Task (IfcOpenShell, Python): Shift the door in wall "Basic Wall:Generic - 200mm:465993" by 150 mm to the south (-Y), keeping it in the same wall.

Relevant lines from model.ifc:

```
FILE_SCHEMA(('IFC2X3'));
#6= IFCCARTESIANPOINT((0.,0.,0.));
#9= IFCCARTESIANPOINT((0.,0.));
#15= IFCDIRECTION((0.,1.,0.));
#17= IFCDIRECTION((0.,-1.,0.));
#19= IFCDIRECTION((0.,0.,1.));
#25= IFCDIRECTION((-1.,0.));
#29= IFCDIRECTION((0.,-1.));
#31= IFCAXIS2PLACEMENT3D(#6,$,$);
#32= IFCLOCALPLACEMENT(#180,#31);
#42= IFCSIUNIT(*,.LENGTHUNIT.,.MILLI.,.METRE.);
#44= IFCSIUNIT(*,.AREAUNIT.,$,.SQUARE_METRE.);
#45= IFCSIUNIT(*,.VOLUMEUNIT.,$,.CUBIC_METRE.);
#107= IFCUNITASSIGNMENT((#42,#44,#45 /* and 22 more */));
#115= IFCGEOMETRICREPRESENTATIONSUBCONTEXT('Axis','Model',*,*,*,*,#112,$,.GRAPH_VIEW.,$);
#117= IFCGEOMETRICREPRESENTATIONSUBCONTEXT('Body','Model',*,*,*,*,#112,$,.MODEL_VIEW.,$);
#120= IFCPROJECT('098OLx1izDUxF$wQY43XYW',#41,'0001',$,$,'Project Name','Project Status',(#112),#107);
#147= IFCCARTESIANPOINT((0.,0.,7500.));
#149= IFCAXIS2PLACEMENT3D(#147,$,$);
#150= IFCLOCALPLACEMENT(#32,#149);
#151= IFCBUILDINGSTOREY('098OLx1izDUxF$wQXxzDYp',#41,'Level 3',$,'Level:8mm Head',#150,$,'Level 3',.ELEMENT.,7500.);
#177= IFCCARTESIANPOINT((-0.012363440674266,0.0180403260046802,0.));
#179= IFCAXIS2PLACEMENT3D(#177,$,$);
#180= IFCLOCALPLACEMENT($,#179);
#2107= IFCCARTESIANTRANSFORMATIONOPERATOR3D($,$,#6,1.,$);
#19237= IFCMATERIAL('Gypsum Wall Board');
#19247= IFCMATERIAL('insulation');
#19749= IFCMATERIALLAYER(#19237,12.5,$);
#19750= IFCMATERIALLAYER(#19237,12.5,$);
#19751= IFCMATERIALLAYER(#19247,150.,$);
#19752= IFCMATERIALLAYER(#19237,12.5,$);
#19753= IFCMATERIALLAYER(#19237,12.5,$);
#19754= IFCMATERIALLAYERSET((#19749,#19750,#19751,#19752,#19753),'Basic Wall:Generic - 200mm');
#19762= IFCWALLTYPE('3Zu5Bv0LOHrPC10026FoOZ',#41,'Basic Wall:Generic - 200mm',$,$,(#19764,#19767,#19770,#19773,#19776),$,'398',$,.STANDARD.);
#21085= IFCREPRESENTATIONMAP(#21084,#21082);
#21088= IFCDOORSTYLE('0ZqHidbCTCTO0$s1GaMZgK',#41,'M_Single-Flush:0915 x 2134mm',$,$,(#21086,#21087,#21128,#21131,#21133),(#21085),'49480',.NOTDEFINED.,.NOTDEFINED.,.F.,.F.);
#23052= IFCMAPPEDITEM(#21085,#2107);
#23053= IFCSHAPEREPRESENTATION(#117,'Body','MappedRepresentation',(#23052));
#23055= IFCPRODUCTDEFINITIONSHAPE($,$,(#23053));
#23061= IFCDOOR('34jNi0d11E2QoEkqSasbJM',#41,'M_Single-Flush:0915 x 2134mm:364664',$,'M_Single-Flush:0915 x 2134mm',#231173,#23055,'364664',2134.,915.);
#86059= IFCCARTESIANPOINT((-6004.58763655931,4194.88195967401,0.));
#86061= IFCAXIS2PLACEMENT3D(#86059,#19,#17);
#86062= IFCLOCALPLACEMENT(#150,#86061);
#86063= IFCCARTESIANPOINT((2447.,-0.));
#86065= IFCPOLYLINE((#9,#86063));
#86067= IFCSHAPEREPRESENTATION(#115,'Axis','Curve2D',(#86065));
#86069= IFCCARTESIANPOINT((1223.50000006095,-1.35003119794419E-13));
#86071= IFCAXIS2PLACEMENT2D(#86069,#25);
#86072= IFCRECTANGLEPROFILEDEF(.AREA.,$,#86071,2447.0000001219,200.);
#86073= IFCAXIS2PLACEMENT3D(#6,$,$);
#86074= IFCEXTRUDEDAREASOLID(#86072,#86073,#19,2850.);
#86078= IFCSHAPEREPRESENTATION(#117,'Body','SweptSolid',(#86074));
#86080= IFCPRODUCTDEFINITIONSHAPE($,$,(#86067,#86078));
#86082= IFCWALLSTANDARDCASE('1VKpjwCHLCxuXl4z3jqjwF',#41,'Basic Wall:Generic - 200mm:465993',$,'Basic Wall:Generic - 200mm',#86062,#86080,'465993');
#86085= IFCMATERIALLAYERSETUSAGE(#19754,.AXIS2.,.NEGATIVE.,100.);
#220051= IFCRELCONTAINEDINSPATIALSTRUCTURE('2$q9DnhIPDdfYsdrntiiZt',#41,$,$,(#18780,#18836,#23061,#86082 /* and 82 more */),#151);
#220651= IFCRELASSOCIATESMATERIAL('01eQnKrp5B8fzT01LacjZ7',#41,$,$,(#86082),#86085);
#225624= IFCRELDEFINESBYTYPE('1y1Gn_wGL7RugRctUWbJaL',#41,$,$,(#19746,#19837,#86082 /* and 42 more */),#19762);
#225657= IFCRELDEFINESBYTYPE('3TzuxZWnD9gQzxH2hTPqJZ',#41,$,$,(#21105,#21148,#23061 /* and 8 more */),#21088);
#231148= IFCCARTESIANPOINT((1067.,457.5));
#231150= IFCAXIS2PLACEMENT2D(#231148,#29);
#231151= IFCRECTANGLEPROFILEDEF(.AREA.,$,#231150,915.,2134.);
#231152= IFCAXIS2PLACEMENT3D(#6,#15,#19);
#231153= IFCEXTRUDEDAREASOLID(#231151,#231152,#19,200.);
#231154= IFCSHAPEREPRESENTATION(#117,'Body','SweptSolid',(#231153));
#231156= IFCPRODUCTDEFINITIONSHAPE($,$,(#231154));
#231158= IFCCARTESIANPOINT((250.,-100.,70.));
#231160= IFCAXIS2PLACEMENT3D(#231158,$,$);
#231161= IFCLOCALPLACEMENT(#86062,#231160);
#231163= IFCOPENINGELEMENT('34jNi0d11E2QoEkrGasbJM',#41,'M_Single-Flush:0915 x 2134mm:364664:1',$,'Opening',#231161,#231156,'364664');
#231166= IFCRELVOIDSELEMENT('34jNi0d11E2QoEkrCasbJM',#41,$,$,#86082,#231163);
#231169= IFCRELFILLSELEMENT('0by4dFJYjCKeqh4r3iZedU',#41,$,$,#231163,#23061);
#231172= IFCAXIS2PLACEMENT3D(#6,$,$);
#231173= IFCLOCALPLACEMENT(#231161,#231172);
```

```python
import ifcopenshell
import ifcopenshell.api.geometry
import ifcopenshell.util.placement
import ifcopenshell.util.unit

model = ifcopenshell.open("model.ifc")
unit_scale = ifcopenshell.util.unit.calculate_unit_scale(model)

door = model.by_guid("34jNi0d11E2QoEkqSasbJM")
opening = door.FillsVoids[0].RelatingOpeningElement
wall = opening.VoidsElements[0].RelatingBuildingElement

wall_matrix = ifcopenshell.util.placement.get_local_placement(wall.ObjectPlacement)
shift = wall_matrix[:3, 0] * 0.15 / unit_scale
before = ifcopenshell.util.placement.get_local_placement(door.ObjectPlacement)[:3, 3].copy()

# The door is placed relative to its opening, so it follows when the opening moves.
matrix = ifcopenshell.util.placement.get_local_placement(opening.ObjectPlacement)
matrix[:3, 3] += shift
ifcopenshell.api.geometry.edit_object_placement(
    model, product=opening, matrix=matrix, is_si=False, should_transform_children=True
)

after = ifcopenshell.util.placement.get_local_placement(door.ObjectPlacement)[:3, 3]
print("door moved by", (after - before).round(3) + 0.0)

model.write("model_edited.ifc")
```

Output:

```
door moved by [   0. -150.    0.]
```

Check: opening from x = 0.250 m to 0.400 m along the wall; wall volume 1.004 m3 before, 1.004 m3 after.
